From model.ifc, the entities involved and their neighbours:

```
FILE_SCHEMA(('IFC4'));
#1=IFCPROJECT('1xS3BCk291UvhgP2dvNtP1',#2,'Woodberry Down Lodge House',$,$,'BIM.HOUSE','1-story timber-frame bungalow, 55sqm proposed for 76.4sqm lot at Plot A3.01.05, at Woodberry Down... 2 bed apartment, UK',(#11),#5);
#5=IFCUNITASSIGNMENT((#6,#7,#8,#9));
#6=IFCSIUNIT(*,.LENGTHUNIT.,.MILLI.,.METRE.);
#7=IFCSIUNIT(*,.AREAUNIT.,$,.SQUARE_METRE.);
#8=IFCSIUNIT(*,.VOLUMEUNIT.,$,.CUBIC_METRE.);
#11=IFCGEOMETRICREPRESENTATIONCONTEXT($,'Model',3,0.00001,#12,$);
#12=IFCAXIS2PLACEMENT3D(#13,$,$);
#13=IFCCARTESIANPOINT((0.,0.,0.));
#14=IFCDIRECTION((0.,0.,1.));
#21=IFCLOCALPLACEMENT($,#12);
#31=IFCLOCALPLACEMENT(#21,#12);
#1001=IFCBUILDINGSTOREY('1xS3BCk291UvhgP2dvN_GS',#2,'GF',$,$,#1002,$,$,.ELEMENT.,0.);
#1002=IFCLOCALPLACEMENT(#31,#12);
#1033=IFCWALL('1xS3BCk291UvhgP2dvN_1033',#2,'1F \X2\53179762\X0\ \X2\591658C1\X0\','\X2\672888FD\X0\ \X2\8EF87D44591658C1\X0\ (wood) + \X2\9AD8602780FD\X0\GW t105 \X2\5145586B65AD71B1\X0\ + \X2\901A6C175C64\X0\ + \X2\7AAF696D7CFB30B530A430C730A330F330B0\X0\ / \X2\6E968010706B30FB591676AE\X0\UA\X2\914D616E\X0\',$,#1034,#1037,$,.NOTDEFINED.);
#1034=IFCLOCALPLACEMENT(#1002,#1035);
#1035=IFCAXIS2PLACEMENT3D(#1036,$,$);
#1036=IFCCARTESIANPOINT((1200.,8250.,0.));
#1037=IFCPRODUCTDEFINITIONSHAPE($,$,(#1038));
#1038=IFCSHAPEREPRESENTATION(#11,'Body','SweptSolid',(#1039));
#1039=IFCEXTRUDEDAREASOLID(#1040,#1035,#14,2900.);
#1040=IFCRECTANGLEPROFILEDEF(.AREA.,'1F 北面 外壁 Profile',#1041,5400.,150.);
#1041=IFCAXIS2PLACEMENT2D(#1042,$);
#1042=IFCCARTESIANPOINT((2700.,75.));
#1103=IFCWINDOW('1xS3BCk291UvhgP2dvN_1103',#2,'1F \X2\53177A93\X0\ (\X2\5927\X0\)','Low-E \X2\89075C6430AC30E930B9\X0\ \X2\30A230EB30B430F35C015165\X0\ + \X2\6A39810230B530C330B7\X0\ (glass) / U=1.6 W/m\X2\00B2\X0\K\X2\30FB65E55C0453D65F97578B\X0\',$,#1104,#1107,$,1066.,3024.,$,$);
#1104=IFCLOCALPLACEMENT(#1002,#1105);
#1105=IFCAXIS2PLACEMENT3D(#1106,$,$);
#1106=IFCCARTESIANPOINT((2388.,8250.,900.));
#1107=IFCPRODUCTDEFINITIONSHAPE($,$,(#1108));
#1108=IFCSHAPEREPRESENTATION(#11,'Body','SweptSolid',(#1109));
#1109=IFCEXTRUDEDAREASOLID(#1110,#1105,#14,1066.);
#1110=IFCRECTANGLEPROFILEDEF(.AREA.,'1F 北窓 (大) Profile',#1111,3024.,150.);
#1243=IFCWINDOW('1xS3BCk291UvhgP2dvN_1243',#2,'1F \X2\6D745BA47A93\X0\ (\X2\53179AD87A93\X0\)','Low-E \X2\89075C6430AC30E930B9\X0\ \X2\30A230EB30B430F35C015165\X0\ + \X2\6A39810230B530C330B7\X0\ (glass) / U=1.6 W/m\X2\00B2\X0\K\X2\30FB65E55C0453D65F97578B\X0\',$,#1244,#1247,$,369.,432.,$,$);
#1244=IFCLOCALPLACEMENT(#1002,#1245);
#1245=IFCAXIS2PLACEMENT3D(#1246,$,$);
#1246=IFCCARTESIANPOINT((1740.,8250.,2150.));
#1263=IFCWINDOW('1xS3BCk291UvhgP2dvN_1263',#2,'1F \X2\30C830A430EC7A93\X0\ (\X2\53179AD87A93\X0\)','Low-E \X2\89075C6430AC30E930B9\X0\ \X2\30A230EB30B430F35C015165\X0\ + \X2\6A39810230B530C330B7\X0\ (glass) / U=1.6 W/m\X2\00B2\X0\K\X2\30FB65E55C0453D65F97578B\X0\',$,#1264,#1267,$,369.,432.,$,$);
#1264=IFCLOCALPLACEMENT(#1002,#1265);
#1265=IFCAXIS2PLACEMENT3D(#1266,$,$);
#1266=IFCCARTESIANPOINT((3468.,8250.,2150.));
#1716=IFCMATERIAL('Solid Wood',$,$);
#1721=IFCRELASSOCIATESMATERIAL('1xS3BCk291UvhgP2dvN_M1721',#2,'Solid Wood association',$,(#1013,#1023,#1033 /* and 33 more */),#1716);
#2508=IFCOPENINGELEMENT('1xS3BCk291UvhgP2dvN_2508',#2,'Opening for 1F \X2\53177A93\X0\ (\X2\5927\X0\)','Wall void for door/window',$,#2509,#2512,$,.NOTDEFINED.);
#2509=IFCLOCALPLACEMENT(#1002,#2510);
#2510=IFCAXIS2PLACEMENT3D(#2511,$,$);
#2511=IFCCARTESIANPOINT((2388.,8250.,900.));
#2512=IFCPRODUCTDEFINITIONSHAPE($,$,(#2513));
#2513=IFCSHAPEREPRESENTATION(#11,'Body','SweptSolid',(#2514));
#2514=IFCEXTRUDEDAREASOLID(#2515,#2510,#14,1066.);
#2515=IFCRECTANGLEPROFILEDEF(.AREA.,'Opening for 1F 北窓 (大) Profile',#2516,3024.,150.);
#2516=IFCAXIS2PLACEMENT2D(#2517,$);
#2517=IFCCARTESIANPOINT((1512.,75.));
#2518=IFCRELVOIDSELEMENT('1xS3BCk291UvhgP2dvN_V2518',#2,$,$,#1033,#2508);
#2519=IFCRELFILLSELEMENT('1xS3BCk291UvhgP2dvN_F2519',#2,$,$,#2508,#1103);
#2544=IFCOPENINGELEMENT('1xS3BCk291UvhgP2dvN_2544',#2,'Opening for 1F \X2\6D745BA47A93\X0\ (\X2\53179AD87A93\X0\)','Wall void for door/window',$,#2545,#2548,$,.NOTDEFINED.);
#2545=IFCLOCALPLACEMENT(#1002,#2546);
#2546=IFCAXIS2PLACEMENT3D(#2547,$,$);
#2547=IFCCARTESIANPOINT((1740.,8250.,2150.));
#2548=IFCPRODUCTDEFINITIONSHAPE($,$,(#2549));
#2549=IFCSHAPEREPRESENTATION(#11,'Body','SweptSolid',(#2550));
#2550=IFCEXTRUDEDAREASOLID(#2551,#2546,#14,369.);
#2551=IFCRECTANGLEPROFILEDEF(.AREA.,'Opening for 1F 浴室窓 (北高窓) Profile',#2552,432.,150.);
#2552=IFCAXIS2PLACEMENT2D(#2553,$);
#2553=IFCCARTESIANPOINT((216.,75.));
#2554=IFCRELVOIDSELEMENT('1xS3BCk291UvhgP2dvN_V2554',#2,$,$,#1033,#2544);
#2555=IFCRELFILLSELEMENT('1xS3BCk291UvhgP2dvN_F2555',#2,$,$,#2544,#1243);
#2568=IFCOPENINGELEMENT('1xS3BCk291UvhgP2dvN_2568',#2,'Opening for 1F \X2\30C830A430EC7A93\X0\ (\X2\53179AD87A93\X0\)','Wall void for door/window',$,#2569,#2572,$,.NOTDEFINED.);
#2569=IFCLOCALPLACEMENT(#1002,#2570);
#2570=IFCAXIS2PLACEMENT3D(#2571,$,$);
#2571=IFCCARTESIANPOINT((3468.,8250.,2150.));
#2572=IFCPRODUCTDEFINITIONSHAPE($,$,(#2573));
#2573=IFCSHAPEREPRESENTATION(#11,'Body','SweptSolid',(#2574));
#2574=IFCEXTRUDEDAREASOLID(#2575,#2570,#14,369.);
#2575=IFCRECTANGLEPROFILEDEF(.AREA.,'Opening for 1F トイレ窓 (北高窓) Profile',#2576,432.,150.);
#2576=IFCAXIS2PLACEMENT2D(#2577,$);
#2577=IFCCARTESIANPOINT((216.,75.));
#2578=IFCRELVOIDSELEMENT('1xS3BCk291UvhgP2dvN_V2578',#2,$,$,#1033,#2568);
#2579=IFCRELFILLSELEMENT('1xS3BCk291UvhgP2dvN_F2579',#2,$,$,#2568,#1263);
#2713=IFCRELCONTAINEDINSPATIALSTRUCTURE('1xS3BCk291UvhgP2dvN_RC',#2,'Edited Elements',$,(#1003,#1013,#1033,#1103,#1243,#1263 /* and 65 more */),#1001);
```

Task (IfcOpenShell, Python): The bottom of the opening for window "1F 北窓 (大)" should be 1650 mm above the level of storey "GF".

```python
import numpy as np
import ifcopenshell
import ifcopenshell.api.geometry
import ifcopenshell.geom
import ifcopenshell.util.element
import ifcopenshell.util.placement
import ifcopenshell.util.shape
import ifcopenshell.util.unit

model = ifcopenshell.open("model.ifc")
unit_scale = ifcopenshell.util.unit.calculate_unit_scale(model)

window = model.by_id(1103)
opening = window.FillsVoids[0].RelatingOpeningElement
storey = ifcopenshell.util.element.get_container(window, ifc_class="IfcBuildingStorey")
level = ifcopenshell.util.placement.get_local_placement(storey.ObjectPlacement)[2, 3]

# The opening's origin need not be at the sill, so measure its lowest point.
shape = ifcopenshell.geom.create_shape(ifcopenshell.geom.settings(), opening)
bottom = ifcopenshell.util.shape.get_shape_bottom_elevation(shape, shape.geometry) / unit_scale
dz = level + 1.65 / unit_scale - bottom

shift = np.array([0.0, 0.0, dz])
# The window is not placed relative to its opening, so move both.
for product in (opening, window):
    matrix = ifcopenshell.util.placement.get_local_placement(product.ObjectPlacement)
    matrix[:3, 3] += shift
    ifcopenshell.api.geometry.edit_object_placement(model, product=product, matrix=matrix, is_si=False)

print(f"moved by {dz * unit_scale:+.3f} m")

model.write("model_updated.ifc")
```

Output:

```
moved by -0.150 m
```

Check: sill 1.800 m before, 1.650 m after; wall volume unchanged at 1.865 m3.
